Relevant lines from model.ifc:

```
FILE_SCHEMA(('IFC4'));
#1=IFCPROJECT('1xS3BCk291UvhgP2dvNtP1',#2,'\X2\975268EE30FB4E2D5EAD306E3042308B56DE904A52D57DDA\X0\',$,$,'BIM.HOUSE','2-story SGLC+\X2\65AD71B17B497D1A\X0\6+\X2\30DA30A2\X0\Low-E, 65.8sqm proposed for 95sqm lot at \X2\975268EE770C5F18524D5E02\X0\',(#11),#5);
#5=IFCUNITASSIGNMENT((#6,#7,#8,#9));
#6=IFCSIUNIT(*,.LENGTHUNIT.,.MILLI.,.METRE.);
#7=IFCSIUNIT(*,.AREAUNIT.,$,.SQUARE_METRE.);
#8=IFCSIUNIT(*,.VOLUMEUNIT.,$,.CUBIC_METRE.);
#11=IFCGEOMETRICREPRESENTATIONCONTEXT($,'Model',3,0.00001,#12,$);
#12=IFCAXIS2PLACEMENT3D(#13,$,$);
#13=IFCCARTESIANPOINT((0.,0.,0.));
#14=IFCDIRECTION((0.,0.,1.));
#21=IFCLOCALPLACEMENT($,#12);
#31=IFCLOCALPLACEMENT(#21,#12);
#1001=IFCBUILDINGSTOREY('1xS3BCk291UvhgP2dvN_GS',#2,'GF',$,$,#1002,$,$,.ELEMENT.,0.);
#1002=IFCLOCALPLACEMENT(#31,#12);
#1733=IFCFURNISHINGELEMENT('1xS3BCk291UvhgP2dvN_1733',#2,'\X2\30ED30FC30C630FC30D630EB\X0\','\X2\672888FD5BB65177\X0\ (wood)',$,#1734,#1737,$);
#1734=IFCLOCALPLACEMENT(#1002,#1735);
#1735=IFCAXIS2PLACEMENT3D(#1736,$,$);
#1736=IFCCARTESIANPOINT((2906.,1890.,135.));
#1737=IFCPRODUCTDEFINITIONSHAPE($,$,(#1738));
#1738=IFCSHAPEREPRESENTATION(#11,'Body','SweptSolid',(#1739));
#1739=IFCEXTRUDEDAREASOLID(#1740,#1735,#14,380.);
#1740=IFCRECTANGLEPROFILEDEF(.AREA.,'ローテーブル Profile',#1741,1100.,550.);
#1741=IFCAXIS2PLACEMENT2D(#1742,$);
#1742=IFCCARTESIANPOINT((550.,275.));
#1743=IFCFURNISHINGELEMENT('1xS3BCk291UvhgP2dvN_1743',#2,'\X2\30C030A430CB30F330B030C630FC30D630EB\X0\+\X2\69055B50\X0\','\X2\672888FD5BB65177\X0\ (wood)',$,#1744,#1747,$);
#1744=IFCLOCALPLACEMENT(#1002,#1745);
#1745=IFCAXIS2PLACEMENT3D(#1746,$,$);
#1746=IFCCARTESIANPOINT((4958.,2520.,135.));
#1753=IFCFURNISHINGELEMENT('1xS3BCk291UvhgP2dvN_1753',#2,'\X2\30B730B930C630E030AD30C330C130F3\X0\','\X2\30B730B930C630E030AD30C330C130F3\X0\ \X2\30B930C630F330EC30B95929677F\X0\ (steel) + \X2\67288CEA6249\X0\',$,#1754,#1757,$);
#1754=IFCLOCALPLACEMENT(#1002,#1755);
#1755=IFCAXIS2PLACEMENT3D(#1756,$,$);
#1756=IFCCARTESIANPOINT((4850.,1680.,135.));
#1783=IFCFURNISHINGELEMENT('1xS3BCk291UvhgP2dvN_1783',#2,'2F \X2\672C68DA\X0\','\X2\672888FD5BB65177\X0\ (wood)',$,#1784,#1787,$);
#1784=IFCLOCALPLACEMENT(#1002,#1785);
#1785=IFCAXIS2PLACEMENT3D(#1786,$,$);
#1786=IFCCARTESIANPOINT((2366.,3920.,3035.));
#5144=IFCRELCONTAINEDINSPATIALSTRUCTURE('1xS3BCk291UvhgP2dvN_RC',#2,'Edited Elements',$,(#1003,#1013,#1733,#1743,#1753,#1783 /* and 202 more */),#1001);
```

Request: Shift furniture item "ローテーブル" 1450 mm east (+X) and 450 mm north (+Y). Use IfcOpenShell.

```python
import ifcopenshell
import ifcopenshell.api.geometry
import ifcopenshell.util.placement

model = ifcopenshell.open("model.ifc")

item = model.by_id(1733)
matrix = ifcopenshell.util.placement.get_local_placement(item.ObjectPlacement)
matrix[0, 3] += 1450.0
matrix[1, 3] += 450.0
ifcopenshell.api.geometry.edit_object_placement(model, product=item, matrix=matrix, is_si=False)

print(ifcopenshell.util.placement.get_local_placement(item.ObjectPlacement).round(3) + 0.0)

model.write("model_rev.ifc")
```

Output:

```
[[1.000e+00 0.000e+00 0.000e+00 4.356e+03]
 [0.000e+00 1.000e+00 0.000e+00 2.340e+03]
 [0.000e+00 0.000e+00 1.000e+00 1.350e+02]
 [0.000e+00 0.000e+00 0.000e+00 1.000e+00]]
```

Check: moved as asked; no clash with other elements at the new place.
